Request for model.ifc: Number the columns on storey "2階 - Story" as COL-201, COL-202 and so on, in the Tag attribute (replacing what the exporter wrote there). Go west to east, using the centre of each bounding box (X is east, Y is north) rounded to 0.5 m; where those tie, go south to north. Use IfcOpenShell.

First a look at what the model holds.

```python
import ifcopenshell
import ifcopenshell.util.element
import ifcopenshell.util.placement

model = ifcopenshell.open("model.ifc")
print(model.schema)
storey = next(s for s in model.by_type("IfcBuildingStorey") if s.Name == "2階 - Story")
columns = [e for e in ifcopenshell.util.element.get_decomposition(storey) if e.is_a("IfcColumn")]
for e in sorted(columns, key=lambda e: e.id()):
    origin = ifcopenshell.util.placement.get_local_placement(e.ObjectPlacement)[:3, 3]
    print(e.id(), e.Tag, e.Name, origin.round(2) + 0.0, sep=" | ")
```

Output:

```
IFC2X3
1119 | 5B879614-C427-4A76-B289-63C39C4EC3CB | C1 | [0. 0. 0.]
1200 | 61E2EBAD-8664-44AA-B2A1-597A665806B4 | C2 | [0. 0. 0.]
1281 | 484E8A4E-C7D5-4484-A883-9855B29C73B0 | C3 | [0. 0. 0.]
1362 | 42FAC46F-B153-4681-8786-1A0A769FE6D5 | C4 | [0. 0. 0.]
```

```python
import ifcopenshell
import ifcopenshell.geom
import ifcopenshell.util.element
import ifcopenshell.util.shape

model = ifcopenshell.open("model.ifc")
settings = ifcopenshell.geom.settings()
settings.set("use-world-coords", True)


def centre(element):
    shape = ifcopenshell.geom.create_shape(settings, element)
    return ifcopenshell.util.shape.get_bbox_centroid(shape.geometry)


storey = next(s for s in model.by_type("IfcBuildingStorey") if s.Name == "2階 - Story")
columns = [e for e in ifcopenshell.util.element.get_decomposition(storey) if e.is_a("IfcColumn")]

# Insertion points can sit at a corner or the storey origin, so sort by the geometry (in metres).
centres = {e: centre(e) for e in columns}
columns.sort(key=lambda e: (round(centres[e][0] / 0.5), centres[e][1]))

for i, e in enumerate(columns, start=1):
    number = f"COL-2{i:02d}"
    e.Tag = number
    print(e.id(), number)

model.write("model_updated.ifc")
```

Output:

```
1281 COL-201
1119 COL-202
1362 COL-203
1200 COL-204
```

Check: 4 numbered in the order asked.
